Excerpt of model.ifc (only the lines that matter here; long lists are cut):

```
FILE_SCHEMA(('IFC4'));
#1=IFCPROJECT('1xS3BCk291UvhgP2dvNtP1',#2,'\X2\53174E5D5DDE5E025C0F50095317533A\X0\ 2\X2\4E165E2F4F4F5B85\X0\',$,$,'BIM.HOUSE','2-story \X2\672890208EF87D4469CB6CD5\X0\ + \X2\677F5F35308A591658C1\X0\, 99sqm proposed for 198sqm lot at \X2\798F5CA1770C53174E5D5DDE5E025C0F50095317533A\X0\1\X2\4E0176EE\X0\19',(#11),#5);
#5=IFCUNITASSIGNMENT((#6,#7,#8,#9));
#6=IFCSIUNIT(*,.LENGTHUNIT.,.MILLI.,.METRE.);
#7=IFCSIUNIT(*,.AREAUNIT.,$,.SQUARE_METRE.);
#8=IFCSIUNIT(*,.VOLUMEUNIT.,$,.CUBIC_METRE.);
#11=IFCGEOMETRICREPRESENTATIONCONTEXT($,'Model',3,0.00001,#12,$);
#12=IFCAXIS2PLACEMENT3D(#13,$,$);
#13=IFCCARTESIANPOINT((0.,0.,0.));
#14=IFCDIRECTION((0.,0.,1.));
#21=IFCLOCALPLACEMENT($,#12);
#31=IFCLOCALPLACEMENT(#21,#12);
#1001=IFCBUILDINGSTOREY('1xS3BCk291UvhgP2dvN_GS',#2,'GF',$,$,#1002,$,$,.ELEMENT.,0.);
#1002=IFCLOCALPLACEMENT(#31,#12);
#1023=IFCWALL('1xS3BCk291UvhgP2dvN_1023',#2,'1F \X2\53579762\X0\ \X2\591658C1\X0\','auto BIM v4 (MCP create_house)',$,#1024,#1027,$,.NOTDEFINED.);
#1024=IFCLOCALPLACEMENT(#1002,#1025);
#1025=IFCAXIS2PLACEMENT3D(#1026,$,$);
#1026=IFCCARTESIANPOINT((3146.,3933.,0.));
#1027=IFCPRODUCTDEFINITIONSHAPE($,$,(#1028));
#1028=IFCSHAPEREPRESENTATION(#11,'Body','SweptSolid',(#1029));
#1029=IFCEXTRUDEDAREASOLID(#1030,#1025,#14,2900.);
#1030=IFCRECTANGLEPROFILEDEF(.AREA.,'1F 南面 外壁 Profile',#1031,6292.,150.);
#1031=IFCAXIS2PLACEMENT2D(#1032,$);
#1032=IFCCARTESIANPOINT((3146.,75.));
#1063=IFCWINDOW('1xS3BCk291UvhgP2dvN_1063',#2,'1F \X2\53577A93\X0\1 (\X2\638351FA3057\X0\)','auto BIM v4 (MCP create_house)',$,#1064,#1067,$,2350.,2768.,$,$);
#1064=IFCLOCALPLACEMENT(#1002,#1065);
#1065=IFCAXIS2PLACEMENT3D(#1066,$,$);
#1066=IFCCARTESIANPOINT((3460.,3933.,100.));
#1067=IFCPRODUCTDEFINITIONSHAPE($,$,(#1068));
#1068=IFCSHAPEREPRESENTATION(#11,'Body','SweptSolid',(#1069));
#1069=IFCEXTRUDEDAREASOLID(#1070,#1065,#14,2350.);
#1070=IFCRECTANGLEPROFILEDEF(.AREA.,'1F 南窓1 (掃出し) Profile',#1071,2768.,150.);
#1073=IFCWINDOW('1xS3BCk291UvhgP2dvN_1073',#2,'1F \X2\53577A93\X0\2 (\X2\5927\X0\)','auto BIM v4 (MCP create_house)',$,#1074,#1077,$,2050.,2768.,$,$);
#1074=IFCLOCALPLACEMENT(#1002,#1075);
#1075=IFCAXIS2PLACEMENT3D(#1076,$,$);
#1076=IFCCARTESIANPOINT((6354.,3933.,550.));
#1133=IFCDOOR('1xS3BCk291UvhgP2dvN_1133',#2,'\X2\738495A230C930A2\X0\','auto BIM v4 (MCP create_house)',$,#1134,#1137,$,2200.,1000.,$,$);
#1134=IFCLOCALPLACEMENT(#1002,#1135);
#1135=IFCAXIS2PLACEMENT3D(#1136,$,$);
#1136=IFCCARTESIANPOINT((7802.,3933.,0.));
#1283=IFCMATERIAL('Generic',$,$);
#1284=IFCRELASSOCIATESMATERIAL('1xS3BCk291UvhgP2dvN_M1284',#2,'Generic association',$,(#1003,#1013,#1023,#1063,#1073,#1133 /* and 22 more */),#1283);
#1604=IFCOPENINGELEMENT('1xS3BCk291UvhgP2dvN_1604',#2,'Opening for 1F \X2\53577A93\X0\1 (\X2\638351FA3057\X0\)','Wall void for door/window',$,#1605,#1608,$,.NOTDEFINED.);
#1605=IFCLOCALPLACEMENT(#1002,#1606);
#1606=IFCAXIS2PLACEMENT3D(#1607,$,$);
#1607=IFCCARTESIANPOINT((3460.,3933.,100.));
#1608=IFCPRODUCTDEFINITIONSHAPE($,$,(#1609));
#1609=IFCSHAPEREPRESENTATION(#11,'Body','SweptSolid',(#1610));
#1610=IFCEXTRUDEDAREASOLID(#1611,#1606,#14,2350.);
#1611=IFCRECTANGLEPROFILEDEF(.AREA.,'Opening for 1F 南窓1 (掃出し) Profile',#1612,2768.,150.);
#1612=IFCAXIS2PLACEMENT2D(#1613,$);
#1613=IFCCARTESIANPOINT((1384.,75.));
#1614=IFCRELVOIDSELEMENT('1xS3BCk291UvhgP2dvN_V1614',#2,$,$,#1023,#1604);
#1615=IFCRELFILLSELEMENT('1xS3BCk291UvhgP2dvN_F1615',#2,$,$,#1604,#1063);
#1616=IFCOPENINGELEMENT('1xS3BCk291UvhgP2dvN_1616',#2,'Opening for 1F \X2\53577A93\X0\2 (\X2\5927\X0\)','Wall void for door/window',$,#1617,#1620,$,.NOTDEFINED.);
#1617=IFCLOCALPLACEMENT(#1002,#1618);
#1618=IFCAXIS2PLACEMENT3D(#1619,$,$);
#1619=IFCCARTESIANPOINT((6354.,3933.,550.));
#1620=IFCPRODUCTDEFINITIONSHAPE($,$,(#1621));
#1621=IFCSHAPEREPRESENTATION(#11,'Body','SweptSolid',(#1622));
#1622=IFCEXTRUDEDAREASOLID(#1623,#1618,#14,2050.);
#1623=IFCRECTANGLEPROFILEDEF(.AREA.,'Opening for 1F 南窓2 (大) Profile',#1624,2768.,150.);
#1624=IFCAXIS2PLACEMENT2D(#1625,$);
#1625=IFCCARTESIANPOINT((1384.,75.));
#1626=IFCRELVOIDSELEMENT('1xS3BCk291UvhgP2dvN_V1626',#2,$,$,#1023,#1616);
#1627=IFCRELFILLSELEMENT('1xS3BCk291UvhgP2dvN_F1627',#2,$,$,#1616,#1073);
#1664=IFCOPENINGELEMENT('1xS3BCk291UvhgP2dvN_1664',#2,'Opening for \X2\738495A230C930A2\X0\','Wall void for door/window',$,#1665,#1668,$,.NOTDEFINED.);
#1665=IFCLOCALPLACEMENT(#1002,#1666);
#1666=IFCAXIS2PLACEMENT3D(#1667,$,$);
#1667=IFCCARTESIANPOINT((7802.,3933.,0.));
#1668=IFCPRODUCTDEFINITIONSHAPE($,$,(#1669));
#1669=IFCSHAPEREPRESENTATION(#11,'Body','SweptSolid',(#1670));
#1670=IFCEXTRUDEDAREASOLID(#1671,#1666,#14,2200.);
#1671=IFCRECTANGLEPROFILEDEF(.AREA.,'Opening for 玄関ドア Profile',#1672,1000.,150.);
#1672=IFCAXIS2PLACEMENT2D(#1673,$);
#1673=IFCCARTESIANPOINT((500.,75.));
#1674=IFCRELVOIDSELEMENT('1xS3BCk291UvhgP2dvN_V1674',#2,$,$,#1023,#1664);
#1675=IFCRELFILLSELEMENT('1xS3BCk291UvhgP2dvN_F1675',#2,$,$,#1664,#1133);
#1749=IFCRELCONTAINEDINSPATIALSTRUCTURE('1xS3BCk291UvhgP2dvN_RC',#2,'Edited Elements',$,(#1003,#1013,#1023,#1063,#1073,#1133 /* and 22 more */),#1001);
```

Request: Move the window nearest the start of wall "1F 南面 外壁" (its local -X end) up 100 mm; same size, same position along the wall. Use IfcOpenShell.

```python
import numpy as np
import ifcopenshell
import ifcopenshell.api.geometry
import ifcopenshell.util.placement
import ifcopenshell.util.unit

model = ifcopenshell.open("model.ifc")
unit_scale = ifcopenshell.util.unit.calculate_unit_scale(model)

window = model.by_guid("1xS3BCk291UvhgP2dvN_1063")
opening = window.FillsVoids[0].RelatingOpeningElement
dz = 0.1 / unit_scale

shift = np.array([0.0, 0.0, dz])
# The window is not placed relative to its opening, so move both.
for product in (opening, window):
    matrix = ifcopenshell.util.placement.get_local_placement(product.ObjectPlacement)
    matrix[:3, 3] += shift
    ifcopenshell.api.geometry.edit_object_placement(model, product=product, matrix=matrix, is_si=False)

print(f"moved by {dz * unit_scale:+.3f} m")

model.write("model_v2.ifc")
```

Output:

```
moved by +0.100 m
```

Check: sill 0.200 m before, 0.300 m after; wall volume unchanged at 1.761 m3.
